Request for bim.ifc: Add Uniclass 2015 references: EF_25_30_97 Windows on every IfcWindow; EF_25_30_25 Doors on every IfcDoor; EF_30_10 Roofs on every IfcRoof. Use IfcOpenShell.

First a look at what the model holds.

```python
import ifcopenshell

model = ifcopenshell.open("bim.ifc")
print(model.schema)
print("classifications:", [c.Name for c in model.by_type("IfcClassification")])
for ifc_class in ("IfcDoor", "IfcRoof", "IfcStair", "IfcWall", "IfcWindow"):
    print(ifc_class, len(model.by_type(ifc_class)))
```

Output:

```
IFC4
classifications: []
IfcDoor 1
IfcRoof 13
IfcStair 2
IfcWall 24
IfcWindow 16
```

```python
import ifcopenshell
import ifcopenshell.api.classification

model = ifcopenshell.open("bim.ifc")

system = ifcopenshell.api.classification.add_classification(model, classification="Uniclass 2015")

codes = {
    "IfcWindow": ("EF_25_30_97", "Windows"),
    "IfcDoor": ("EF_25_30_25", "Doors"),
    "IfcRoof": ("EF_30_10", "Roofs"),
}
for ifc_class, (code, name) in codes.items():
    products = model.by_type(ifc_class)
    ifcopenshell.api.classification.add_reference(
        model, products=products, classification=system, identification=code, name=name
    )
    print(code, len(products))

model.write("bim_rev.ifc")
```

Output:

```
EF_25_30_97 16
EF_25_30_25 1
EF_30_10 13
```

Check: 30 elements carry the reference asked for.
